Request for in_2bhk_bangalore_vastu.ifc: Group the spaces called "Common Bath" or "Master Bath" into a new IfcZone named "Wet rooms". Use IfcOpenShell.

First a look at what the model holds.

```python
import ifcopenshell

model = ifcopenshell.open("in_2bhk_bangalore_vastu.ifc")
print(model.schema)
seen = {}
for space in model.by_type("IfcSpace"):
    seen[space.LongName] = seen.get(space.LongName, 0) + 1
for name, count in sorted(seen.items(), key=str):
    print(count, "x", name)
print("zones:", [z.Name for z in model.by_type("IfcZone")][:20])
```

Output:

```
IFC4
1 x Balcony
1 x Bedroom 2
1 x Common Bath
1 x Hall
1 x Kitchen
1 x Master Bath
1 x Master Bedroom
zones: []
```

```python
import ifcopenshell
import ifcopenshell.api.group
import ifcopenshell.api.root

model = ifcopenshell.open("in_2bhk_bangalore_vastu.ifc")

names = {"Common Bath", "Master Bath"}
spaces = [s for s in model.by_type("IfcSpace") if s.LongName in names]

zone = ifcopenshell.api.root.create_entity(model, ifc_class="IfcZone", name="Wet rooms")
ifcopenshell.api.group.assign_group(model, products=spaces, group=zone)
print(len(spaces), "spaces in", zone.Name)

model.write("in_2bhk_bangalore_vastu_rev.ifc")
```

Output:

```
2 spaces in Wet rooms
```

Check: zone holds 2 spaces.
